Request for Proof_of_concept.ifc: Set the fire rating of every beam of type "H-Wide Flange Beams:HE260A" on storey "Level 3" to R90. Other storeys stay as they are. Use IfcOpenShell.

First a look at what the model holds.

```python
import ifcopenshell
import ifcopenshell.util.element

model = ifcopenshell.open("Proof_of_concept.ifc")
print(model.schema)
storey = next(s for s in model.by_type("IfcBuildingStorey") if s.Name == "Level 3")
beams = [e for e in ifcopenshell.util.element.get_decomposition(storey) if e.is_a("IfcBeam")]
seen = {}
for e in beams:
    element_type = ifcopenshell.util.element.get_type(e)
    key = (element_type.Name if element_type != e and element_type else None, ifcopenshell.util.element.get_pset(e, "Pset_BeamCommon", "FireRating"))
    seen[key] = seen.get(key, 0) + 1
for (name, value), count in sorted(seen.items(), key=str):
    print(count, "x", name, "|", value)
```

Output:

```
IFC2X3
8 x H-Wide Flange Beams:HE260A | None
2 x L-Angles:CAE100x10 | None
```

```python
import ifcopenshell
import ifcopenshell.api.pset
import ifcopenshell.util.element

model = ifcopenshell.open("Proof_of_concept.ifc")

storey = next(s for s in model.by_type("IfcBuildingStorey") if s.Name == "Level 3")
beams = [e for e in ifcopenshell.util.element.get_decomposition(storey) if e.is_a("IfcBeam")]

count = 0
for e in beams:
    element_type = ifcopenshell.util.element.get_type(e)
    if element_type in (None, e) or element_type.Name != "H-Wide Flange Beams:HE260A":
        continue
    # add_pset returns the element's existing set when there is one.
    pset = ifcopenshell.api.pset.add_pset(model, product=e, name="Pset_BeamCommon")
    ifcopenshell.api.pset.edit_pset(model, pset=pset, properties={"FireRating": "R90"})
    count += 1

print(count, "beams updated")

model.write("Proof_of_concept-out.ifc")
```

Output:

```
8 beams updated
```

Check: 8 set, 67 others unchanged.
